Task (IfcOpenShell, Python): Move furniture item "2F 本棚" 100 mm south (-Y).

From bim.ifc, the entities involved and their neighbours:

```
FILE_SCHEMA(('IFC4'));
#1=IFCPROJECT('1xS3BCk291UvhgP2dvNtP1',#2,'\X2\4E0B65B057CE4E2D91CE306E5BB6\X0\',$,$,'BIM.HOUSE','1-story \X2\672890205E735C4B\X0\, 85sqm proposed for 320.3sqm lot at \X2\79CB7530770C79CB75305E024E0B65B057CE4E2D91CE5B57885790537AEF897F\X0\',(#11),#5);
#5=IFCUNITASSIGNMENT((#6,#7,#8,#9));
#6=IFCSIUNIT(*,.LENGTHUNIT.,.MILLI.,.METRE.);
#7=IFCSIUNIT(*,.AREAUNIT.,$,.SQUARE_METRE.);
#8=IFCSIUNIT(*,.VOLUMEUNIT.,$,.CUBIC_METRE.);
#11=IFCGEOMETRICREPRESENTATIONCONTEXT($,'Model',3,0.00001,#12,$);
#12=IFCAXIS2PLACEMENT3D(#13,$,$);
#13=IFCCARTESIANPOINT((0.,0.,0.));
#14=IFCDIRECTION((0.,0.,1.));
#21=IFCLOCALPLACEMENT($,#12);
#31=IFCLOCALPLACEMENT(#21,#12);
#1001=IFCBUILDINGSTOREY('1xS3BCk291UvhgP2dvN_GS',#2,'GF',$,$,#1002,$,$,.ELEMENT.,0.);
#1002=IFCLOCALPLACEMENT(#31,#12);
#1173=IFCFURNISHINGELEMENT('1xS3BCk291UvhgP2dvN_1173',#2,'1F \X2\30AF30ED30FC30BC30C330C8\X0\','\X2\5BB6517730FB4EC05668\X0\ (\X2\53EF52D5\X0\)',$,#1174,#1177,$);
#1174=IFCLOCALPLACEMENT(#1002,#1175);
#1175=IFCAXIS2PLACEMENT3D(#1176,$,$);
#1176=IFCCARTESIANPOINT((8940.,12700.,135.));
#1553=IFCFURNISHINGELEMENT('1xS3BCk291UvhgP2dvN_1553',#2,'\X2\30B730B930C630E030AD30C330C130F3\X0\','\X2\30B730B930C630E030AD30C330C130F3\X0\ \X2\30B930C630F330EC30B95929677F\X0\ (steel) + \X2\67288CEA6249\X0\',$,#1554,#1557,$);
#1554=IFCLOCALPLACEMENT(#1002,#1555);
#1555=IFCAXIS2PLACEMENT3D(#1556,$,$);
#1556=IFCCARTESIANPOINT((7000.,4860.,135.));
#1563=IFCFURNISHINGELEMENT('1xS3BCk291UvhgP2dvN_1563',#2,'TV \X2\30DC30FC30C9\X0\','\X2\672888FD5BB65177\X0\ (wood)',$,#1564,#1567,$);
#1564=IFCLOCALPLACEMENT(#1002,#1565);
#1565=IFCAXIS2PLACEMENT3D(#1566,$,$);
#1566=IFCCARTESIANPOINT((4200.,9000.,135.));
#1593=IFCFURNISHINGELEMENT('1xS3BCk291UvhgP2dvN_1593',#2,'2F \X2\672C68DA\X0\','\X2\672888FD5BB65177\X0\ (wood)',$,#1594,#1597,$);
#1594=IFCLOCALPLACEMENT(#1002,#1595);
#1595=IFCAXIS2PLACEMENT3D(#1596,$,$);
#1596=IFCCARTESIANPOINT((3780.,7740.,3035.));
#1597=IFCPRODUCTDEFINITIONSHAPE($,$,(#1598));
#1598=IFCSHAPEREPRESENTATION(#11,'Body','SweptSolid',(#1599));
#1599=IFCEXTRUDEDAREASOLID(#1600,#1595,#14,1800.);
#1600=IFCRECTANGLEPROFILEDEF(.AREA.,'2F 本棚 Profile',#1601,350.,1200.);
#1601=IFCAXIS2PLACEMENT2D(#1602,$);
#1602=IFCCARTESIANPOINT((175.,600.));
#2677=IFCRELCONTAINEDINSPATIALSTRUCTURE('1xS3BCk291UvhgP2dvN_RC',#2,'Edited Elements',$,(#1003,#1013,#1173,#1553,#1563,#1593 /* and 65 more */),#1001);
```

```python
import ifcopenshell
import ifcopenshell.api.geometry
import ifcopenshell.util.placement
import ifcopenshell.util.unit

model = ifcopenshell.open("bim.ifc")
unit_scale = ifcopenshell.util.unit.calculate_unit_scale(model)

item = model.by_id(1593)
matrix = ifcopenshell.util.placement.get_local_placement(item.ObjectPlacement)
matrix[1, 3] -= 0.1 / unit_scale
ifcopenshell.api.geometry.edit_object_placement(model, product=item, matrix=matrix, is_si=False)

print(ifcopenshell.util.placement.get_local_placement(item.ObjectPlacement).round(3) + 0.0)

model.write("bim_v2.ifc")
```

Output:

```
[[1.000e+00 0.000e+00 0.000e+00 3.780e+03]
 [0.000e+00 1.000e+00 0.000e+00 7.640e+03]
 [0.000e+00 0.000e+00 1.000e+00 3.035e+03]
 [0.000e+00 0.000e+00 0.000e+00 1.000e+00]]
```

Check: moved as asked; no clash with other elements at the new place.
